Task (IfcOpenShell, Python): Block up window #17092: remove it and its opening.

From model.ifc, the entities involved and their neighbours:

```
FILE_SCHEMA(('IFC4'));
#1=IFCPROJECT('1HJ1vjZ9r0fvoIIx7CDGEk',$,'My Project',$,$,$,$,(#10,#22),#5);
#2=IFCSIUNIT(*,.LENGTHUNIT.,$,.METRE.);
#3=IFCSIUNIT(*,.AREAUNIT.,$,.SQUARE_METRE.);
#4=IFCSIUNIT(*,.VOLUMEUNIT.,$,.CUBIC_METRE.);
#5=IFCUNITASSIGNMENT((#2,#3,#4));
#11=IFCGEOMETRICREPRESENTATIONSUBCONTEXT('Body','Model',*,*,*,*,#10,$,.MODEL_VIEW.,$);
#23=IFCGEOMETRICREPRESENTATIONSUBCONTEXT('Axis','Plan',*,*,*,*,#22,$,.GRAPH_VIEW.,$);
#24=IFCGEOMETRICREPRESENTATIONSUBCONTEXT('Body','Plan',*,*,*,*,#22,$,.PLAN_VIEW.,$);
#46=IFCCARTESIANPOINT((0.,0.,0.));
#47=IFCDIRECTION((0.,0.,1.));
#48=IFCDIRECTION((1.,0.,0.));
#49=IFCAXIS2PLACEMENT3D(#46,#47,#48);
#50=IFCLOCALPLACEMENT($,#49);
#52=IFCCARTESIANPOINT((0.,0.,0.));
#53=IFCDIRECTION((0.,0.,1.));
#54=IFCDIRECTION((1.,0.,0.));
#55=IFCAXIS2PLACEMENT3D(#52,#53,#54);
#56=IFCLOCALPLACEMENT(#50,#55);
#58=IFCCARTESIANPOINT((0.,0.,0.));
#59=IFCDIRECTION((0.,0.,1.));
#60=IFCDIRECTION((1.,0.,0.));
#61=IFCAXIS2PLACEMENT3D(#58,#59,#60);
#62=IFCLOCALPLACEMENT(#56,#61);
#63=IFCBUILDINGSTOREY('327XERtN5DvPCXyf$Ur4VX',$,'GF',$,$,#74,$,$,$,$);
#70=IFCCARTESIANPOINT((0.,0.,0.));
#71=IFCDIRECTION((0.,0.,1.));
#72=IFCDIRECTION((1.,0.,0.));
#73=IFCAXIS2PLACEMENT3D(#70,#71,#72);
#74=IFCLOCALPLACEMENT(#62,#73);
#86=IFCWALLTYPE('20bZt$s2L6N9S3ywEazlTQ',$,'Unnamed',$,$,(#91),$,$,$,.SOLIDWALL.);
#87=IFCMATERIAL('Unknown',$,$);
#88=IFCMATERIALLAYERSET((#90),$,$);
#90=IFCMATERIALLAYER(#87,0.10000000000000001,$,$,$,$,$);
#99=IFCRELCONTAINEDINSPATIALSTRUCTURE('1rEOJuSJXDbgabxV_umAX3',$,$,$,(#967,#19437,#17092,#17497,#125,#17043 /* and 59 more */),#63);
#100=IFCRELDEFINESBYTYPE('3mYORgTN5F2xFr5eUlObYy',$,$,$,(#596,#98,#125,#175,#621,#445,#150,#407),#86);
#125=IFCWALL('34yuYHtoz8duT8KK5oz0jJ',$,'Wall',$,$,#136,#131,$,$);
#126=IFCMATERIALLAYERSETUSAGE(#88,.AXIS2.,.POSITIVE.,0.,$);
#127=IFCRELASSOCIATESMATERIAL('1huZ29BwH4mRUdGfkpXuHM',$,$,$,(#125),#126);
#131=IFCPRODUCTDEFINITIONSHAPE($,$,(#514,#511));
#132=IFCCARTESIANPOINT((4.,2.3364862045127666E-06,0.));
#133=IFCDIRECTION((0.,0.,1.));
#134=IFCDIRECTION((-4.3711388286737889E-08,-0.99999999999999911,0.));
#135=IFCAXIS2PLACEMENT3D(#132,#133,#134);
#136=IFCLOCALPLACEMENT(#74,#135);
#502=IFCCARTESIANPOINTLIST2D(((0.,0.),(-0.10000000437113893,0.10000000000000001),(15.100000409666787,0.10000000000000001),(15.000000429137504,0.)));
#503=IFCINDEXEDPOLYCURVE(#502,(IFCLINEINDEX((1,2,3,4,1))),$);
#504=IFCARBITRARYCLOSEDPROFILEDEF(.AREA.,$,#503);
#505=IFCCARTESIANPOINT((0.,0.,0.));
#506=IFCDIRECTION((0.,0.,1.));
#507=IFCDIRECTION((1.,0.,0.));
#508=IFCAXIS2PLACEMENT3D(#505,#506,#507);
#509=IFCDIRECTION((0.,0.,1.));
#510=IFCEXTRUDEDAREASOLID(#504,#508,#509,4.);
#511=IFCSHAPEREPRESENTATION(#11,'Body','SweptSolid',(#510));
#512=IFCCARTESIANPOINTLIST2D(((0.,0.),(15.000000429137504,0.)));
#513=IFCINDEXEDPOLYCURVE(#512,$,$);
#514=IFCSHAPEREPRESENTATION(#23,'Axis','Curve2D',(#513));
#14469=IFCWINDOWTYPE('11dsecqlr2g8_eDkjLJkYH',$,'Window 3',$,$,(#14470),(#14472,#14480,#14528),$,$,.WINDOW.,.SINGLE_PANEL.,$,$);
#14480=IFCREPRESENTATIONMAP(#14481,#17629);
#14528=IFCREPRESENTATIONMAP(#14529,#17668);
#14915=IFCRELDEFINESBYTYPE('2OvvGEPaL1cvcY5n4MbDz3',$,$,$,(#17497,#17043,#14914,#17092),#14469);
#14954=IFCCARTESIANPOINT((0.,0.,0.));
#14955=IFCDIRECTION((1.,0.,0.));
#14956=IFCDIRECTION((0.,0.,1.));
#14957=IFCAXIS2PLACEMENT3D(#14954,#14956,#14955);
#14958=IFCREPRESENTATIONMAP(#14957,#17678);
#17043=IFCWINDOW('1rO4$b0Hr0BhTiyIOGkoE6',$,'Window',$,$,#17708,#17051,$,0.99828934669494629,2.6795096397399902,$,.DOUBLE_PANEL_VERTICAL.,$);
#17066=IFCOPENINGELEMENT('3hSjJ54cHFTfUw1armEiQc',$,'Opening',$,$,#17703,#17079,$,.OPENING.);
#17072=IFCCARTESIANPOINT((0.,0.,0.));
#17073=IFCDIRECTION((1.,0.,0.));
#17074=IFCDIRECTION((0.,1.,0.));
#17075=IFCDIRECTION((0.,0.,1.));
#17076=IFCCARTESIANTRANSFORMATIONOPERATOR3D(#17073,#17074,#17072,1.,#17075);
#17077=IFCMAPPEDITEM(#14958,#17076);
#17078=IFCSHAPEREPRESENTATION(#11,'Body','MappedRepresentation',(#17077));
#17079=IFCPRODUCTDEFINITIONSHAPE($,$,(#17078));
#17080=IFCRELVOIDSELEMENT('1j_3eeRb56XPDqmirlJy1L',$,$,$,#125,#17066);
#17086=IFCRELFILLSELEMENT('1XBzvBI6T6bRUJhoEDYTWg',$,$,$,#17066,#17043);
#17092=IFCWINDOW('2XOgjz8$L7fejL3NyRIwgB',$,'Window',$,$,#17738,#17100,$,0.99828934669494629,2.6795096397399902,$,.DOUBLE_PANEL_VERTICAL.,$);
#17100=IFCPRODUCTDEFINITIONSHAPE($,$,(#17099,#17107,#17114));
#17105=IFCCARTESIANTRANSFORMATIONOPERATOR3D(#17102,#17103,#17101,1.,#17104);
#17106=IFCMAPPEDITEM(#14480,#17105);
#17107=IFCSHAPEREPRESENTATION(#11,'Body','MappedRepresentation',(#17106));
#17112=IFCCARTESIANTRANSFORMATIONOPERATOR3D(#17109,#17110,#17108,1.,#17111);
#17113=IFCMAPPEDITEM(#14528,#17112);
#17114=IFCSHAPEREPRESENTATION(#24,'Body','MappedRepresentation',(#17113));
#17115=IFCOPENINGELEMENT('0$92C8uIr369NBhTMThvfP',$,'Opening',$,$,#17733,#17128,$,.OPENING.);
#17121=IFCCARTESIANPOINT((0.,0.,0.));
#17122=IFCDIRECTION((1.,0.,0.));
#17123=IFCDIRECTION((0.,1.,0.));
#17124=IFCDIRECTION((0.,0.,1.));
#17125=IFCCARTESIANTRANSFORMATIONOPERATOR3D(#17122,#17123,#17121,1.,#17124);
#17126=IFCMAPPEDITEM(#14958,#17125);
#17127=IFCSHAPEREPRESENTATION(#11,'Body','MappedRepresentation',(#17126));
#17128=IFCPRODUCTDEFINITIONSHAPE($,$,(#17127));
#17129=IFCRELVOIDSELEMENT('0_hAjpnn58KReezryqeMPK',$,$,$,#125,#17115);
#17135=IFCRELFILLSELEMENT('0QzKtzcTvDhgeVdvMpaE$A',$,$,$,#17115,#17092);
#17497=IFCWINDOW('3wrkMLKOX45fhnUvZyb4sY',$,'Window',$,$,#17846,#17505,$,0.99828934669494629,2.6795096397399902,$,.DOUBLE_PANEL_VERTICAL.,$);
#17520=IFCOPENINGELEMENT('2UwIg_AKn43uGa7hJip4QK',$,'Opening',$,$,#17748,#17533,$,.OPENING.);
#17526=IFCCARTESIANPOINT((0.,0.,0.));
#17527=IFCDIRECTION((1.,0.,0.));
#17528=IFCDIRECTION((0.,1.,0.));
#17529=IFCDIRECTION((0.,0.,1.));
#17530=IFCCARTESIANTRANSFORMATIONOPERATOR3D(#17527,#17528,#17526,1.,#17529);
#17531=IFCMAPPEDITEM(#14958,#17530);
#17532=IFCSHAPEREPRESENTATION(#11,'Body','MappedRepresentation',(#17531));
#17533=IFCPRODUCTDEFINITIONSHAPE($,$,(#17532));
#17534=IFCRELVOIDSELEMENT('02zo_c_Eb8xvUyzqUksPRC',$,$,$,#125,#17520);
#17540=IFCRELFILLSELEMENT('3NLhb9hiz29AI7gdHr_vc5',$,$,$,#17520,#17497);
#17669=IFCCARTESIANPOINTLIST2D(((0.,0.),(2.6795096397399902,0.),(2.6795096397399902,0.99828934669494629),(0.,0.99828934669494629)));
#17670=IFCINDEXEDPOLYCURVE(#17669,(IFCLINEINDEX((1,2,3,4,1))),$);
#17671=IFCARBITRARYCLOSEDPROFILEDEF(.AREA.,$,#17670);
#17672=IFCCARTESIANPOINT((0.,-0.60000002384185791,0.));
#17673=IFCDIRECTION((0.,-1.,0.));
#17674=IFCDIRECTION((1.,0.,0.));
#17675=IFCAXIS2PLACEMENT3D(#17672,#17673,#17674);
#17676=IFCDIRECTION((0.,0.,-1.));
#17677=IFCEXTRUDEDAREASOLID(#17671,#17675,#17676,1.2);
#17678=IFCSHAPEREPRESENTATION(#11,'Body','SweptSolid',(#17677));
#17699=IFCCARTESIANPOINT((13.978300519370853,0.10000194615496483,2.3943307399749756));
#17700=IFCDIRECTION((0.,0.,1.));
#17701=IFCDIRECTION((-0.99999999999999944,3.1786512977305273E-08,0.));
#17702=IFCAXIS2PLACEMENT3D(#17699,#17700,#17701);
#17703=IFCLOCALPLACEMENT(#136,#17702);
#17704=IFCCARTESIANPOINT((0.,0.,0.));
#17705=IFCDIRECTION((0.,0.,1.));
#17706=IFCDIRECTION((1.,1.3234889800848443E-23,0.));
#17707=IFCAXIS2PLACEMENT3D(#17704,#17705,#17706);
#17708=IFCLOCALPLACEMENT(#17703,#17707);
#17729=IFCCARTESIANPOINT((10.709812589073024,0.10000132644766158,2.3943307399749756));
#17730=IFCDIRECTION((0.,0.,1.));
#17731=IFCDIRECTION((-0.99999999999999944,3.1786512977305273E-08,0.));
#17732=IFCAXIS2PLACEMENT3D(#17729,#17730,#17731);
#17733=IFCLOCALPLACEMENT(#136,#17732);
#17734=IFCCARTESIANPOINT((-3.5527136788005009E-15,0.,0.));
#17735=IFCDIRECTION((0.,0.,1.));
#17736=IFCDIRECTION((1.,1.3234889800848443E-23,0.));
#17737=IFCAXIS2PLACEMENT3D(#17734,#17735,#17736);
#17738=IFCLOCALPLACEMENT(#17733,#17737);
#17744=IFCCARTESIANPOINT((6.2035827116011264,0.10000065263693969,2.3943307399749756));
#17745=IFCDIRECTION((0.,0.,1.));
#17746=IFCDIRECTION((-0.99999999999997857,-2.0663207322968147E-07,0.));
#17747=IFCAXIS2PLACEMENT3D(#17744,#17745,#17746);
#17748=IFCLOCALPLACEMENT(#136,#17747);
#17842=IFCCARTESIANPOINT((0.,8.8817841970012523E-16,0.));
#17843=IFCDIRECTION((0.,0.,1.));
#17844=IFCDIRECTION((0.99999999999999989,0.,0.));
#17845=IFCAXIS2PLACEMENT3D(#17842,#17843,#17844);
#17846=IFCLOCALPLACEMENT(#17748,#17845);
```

```python
import ifcopenshell
import ifcopenshell.api.feature
import ifcopenshell.api.root
import ifcopenshell.geom
import ifcopenshell.util.shape

model = ifcopenshell.open("model.ifc")
settings = ifcopenshell.geom.settings()


def volume(element):
    """Net volume in cubic metres, openings subtracted."""
    shape = ifcopenshell.geom.create_shape(settings, element)
    return ifcopenshell.util.shape.get_volume(shape.geometry)


window = model.by_guid("2XOgjz8$L7fejL3NyRIwgB")
opening = window.FillsVoids[0].RelatingOpeningElement
wall = opening.VoidsElements[0].RelatingBuildingElement
before = volume(wall)

ifcopenshell.api.root.remove_product(model, product=window)
ifcopenshell.api.feature.remove_feature(model, feature=opening)

after = volume(wall)

print(f"wall volume {before:.3f} -> {after:.3f} m3")

model.write("model_edited.ifc")
```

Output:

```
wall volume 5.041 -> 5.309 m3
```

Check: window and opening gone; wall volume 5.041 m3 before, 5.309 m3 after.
